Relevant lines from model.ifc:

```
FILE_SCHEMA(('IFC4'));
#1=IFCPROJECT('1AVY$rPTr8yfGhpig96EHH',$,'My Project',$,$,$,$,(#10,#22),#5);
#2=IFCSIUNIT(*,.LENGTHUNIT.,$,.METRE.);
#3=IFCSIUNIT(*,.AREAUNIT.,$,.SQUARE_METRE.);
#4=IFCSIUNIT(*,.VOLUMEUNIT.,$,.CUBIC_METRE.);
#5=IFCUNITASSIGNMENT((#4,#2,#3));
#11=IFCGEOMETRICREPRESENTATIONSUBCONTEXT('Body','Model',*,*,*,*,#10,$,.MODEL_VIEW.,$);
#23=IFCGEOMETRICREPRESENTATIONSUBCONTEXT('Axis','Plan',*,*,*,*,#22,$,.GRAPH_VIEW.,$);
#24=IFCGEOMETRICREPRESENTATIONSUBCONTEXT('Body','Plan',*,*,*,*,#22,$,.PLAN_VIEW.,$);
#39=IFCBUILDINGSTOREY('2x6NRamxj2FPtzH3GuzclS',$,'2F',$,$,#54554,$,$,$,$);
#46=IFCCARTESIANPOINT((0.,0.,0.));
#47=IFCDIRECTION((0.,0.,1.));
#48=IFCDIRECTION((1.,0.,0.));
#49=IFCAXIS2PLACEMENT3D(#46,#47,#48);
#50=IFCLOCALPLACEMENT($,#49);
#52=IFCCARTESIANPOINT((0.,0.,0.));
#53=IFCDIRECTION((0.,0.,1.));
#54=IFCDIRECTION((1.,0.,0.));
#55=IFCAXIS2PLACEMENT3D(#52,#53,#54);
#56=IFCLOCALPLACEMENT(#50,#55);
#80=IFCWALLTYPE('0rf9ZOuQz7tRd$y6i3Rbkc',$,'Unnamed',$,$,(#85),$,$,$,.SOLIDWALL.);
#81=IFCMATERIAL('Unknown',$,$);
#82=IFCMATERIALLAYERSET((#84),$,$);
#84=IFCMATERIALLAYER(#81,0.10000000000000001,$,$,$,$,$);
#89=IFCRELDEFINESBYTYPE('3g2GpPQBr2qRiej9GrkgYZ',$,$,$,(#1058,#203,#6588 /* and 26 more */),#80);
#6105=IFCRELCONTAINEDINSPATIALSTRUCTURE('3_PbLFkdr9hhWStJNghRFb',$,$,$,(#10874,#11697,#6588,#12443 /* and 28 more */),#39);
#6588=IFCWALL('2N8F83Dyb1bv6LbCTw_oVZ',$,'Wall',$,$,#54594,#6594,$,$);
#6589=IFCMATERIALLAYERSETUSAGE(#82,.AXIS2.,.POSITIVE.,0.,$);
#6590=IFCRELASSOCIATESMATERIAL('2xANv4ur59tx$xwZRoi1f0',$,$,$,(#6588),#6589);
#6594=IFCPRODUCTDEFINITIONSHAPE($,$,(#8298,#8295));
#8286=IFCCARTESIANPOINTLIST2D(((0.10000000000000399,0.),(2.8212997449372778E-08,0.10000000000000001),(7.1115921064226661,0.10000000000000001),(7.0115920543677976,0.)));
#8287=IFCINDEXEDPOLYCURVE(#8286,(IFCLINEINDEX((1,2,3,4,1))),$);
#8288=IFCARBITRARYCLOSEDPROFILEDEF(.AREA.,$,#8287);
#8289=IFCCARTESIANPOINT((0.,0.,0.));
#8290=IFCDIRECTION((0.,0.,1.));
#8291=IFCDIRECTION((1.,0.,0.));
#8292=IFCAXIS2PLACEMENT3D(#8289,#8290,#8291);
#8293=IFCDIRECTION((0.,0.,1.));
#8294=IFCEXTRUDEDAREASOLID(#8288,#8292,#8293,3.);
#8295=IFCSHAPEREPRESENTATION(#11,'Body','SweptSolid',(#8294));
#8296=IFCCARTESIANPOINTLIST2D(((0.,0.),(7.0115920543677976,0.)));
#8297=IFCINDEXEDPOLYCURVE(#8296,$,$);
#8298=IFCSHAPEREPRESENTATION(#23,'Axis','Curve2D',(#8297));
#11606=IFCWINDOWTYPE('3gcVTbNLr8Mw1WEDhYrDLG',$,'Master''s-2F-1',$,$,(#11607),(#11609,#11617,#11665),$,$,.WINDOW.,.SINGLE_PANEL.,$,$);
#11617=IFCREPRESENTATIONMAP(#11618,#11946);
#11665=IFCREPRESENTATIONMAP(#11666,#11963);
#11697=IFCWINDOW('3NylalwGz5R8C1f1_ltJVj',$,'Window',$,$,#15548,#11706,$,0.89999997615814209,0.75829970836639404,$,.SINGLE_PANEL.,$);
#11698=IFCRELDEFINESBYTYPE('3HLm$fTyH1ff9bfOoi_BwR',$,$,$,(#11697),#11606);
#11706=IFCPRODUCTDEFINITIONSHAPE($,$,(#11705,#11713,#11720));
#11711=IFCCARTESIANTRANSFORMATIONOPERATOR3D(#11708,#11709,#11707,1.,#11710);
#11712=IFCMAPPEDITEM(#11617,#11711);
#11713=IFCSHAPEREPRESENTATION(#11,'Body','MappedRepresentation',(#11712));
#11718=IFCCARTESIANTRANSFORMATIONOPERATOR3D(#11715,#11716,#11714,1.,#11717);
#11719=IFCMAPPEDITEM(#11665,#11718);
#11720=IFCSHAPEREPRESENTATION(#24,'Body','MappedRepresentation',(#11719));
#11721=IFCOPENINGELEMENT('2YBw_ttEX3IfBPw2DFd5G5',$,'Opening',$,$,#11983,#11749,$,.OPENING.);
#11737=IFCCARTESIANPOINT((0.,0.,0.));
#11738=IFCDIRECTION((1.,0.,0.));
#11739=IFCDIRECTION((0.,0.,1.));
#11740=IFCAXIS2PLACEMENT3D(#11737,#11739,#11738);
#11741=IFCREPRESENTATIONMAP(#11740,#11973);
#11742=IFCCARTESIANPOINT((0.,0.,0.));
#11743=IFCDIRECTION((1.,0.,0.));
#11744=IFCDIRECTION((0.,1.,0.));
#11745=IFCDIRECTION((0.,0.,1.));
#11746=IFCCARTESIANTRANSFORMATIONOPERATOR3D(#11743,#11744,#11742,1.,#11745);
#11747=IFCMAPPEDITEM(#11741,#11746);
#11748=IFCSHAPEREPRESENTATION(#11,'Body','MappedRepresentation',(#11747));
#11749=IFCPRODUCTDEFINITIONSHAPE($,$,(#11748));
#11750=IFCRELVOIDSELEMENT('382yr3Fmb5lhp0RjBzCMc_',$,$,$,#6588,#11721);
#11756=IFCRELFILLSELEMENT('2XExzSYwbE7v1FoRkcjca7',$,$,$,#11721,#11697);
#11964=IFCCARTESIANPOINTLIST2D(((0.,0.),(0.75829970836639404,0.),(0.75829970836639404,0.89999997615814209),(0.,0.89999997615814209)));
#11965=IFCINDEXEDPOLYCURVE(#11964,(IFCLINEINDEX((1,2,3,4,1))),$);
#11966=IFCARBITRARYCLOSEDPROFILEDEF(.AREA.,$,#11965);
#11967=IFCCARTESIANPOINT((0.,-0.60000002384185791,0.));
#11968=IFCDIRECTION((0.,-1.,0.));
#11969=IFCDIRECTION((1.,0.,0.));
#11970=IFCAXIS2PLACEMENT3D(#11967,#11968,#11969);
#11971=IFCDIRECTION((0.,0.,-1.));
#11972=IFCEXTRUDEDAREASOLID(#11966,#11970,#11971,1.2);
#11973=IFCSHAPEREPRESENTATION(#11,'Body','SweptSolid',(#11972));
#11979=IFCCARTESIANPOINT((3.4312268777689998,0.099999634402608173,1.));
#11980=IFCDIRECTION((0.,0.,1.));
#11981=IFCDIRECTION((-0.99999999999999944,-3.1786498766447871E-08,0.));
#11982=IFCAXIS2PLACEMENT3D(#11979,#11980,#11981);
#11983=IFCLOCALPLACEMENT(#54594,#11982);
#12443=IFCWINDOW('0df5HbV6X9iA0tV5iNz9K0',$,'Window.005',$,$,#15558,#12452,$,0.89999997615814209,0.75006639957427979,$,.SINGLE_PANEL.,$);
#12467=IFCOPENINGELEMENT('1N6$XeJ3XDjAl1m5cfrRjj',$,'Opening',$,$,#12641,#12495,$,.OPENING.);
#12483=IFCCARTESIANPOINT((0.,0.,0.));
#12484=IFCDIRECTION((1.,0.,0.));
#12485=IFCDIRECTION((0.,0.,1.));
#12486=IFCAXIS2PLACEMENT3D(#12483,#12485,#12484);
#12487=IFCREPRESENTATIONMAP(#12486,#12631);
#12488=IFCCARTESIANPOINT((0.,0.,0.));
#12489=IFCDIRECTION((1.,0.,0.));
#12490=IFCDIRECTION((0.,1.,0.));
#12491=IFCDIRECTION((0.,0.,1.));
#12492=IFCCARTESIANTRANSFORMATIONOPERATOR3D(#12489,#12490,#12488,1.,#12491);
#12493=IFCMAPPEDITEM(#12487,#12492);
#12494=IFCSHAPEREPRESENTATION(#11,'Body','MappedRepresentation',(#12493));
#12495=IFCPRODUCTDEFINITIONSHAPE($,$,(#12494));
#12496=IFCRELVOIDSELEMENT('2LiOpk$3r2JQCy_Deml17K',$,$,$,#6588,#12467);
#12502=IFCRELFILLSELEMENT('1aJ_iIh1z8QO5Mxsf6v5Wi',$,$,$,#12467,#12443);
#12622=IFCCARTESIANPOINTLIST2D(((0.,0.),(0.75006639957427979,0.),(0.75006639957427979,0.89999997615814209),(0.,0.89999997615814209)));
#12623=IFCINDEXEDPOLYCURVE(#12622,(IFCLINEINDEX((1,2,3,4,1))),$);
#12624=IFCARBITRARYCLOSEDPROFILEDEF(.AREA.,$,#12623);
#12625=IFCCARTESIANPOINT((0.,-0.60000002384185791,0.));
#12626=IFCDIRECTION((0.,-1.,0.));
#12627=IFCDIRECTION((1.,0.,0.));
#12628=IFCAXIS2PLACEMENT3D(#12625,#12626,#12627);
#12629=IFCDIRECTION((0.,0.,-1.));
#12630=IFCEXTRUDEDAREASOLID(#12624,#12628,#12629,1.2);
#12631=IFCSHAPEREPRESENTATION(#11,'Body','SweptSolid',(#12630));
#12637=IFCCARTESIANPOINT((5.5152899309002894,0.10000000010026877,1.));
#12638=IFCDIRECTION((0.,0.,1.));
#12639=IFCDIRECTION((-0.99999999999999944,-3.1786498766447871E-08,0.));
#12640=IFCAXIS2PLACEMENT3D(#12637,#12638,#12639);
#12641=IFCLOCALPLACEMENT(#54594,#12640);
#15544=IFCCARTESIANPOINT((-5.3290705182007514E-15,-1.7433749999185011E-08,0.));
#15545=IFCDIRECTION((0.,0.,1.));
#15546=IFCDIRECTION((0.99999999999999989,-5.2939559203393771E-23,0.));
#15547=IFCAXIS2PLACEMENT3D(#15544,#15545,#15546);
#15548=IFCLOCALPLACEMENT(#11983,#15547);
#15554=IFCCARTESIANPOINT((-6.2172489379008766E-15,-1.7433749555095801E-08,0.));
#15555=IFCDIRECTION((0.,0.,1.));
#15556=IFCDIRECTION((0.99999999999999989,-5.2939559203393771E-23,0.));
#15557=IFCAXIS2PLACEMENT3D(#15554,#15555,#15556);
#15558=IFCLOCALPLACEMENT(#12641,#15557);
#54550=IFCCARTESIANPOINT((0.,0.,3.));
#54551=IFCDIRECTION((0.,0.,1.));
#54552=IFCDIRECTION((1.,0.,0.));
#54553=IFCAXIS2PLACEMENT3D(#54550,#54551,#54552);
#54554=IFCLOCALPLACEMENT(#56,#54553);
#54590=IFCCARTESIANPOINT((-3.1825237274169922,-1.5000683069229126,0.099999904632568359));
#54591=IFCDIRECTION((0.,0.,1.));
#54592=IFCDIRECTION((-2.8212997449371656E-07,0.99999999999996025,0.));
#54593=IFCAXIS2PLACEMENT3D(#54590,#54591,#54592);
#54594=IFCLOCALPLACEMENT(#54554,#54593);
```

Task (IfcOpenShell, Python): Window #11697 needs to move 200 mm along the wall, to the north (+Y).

```python
import ifcopenshell
import ifcopenshell.api.geometry
import ifcopenshell.util.placement
import ifcopenshell.util.unit

model = ifcopenshell.open("model.ifc")
unit_scale = ifcopenshell.util.unit.calculate_unit_scale(model)

window = model.by_guid("3NylalwGz5R8C1f1_ltJVj")
opening = window.FillsVoids[0].RelatingOpeningElement
wall = opening.VoidsElements[0].RelatingBuildingElement

wall_matrix = ifcopenshell.util.placement.get_local_placement(wall.ObjectPlacement)
shift = wall_matrix[:3, 0] * 0.2 / unit_scale
before = ifcopenshell.util.placement.get_local_placement(window.ObjectPlacement)[:3, 3].copy()

# The window is placed relative to its opening, so it follows when the opening moves.
matrix = ifcopenshell.util.placement.get_local_placement(opening.ObjectPlacement)
matrix[:3, 3] += shift
ifcopenshell.api.geometry.edit_object_placement(
    model, product=opening, matrix=matrix, is_si=False, should_transform_children=True
)

after = ifcopenshell.util.placement.get_local_placement(window.ObjectPlacement)[:3, 3]
print("window moved by", (after - before).round(3) + 0.0)

model.write("model_edited.ifc")
```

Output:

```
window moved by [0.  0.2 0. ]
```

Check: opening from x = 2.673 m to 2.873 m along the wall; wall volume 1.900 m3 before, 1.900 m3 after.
